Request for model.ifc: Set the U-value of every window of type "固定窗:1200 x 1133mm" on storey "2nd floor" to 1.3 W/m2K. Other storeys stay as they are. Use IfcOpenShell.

First a look at what the model holds.

```python
import ifcopenshell
import ifcopenshell.util.element

model = ifcopenshell.open("model.ifc")
print(model.schema)
storey = next(s for s in model.by_type("IfcBuildingStorey") if s.Name == "2nd floor")
windows = [e for e in ifcopenshell.util.element.get_decomposition(storey) if e.is_a("IfcWindow")]
seen = {}
for e in windows:
    element_type = ifcopenshell.util.element.get_type(e)
    key = (element_type.Name if element_type != e and element_type else None, ifcopenshell.util.element.get_pset(e, "Pset_WindowCommon", "ThermalTransmittance"))
    seen[key] = seen.get(key, 0) + 1
for (name, value), count in sorted(seen.items(), key=str):
    print(count, "x", name, "|", value)
```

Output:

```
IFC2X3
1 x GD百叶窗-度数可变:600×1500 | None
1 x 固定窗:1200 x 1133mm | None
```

```python
import ifcopenshell
import ifcopenshell.api.pset
import ifcopenshell.util.element

model = ifcopenshell.open("model.ifc")

storey = next(s for s in model.by_type("IfcBuildingStorey") if s.Name == "2nd floor")
windows = [e for e in ifcopenshell.util.element.get_decomposition(storey) if e.is_a("IfcWindow")]

count = 0
for e in windows:
    element_type = ifcopenshell.util.element.get_type(e)
    if element_type in (None, e) or element_type.Name != "固定窗:1200 x 1133mm":
        continue
    # add_pset returns the element's existing set when there is one.
    pset = ifcopenshell.api.pset.add_pset(model, product=e, name="Pset_WindowCommon")
    ifcopenshell.api.pset.edit_pset(model, pset=pset, properties={"ThermalTransmittance": 1.3})
    count += 1

print(count, "windows updated")

model.write("model_rev.ifc")
```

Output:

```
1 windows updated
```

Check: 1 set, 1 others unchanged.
